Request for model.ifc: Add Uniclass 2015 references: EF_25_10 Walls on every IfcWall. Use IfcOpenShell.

First a look at what the model holds.

```python
import ifcopenshell

model = ifcopenshell.open("model.ifc")
print(model.schema)
print("classifications:", [c.Name for c in model.by_type("IfcClassification")])
for ifc_class in ("IfcDoor", "IfcRoof", "IfcStair", "IfcWall", "IfcWindow"):
    print(ifc_class, len(model.by_type(ifc_class)))
```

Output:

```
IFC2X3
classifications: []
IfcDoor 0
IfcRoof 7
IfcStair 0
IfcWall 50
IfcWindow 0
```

```python
import ifcopenshell
import ifcopenshell.api.classification

model = ifcopenshell.open("model.ifc")

# IFC2X3 requires Source and Edition and has no link from the project to the system.
system = model.create_entity("IfcClassification", Source="NBS", Edition="2015", Name="Uniclass 2015")

codes = {
    "IfcWall": ("EF_25_10", "Walls"),
}
for ifc_class, (code, name) in codes.items():
    products = model.by_type(ifc_class)
    ifcopenshell.api.classification.add_reference(
        model, products=products, classification=system, identification=code, name=name
    )
    print(code, len(products))

model.write("model_rev.ifc")
```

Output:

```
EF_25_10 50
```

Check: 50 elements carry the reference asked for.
